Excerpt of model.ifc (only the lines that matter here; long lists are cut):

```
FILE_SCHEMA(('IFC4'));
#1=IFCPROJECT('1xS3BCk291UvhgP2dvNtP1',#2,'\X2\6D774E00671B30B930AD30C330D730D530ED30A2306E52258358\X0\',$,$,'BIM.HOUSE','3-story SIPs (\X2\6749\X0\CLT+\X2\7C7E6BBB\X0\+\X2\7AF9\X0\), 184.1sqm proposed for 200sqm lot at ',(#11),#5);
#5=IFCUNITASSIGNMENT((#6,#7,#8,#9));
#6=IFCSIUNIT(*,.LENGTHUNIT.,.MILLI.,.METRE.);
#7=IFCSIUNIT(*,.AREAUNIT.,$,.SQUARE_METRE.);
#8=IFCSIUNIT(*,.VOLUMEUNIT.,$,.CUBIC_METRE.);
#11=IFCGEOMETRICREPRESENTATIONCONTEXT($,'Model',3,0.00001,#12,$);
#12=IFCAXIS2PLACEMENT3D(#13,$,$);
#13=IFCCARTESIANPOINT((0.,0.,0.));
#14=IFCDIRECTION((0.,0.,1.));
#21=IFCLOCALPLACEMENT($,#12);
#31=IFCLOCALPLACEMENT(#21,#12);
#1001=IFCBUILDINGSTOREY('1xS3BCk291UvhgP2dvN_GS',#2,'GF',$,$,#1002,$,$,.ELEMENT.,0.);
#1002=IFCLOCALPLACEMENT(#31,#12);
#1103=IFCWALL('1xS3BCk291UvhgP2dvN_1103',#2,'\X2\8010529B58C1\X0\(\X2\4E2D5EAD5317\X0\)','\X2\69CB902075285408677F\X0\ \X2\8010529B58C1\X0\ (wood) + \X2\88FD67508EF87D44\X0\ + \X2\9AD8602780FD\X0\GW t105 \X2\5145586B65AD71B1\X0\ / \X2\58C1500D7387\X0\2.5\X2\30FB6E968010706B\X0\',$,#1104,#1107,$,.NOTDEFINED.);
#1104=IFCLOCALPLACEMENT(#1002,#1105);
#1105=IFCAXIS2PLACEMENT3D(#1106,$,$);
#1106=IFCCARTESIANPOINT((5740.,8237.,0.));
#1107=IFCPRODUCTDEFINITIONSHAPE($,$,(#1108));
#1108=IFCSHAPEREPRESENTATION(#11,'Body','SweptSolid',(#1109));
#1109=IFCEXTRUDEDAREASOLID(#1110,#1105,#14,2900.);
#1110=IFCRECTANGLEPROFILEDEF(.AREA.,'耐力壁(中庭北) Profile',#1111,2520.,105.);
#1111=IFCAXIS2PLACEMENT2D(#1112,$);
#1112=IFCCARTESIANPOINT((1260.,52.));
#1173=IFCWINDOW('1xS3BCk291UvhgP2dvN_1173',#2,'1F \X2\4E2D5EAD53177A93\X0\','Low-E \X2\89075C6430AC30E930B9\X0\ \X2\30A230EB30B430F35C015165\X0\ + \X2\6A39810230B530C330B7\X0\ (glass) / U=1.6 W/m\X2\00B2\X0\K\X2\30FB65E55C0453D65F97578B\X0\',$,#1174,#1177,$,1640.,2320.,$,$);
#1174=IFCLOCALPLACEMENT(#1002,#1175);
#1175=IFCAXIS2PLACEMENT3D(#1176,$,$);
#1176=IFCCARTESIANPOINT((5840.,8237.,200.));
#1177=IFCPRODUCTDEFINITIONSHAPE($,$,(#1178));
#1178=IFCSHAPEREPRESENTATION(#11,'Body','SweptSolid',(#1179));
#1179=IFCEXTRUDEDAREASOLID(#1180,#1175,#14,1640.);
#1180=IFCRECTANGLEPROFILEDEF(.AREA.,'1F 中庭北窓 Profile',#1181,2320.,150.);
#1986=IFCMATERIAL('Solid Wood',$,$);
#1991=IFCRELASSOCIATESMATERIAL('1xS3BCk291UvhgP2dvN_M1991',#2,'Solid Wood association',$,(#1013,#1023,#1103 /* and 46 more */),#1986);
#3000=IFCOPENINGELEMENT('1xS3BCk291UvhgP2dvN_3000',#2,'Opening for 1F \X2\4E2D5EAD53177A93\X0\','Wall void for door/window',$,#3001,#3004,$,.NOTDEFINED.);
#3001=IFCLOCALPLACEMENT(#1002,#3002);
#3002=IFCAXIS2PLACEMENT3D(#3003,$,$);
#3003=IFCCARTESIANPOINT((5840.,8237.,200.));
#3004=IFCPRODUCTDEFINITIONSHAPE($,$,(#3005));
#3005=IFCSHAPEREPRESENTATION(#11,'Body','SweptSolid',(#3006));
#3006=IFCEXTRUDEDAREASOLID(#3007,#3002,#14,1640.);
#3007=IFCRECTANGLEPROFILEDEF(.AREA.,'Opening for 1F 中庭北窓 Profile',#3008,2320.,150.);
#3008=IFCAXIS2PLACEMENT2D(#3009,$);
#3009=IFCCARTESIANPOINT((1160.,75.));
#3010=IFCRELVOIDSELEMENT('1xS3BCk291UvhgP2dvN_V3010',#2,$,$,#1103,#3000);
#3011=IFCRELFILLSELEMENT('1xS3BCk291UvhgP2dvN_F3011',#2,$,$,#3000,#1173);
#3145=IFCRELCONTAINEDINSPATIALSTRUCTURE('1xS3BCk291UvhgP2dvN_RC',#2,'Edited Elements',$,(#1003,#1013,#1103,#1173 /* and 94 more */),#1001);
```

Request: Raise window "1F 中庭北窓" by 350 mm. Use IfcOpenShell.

```python
import numpy as np
import ifcopenshell
import ifcopenshell.api.geometry
import ifcopenshell.util.placement
import ifcopenshell.util.unit

model = ifcopenshell.open("model.ifc")
unit_scale = ifcopenshell.util.unit.calculate_unit_scale(model)

window = model.by_id(1173)
opening = window.FillsVoids[0].RelatingOpeningElement
dz = 350.0

shift = np.array([0.0, 0.0, dz])
# The window is not placed relative to its opening, so move both.
for product in (opening, window):
    matrix = ifcopenshell.util.placement.get_local_placement(product.ObjectPlacement)
    matrix[:3, 3] += shift
    ifcopenshell.api.geometry.edit_object_placement(model, product=product, matrix=matrix, is_si=False)

print(f"moved by {dz * unit_scale:+.3f} m")

model.write("model-out.ifc")
```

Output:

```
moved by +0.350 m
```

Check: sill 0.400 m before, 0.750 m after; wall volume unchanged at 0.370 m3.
